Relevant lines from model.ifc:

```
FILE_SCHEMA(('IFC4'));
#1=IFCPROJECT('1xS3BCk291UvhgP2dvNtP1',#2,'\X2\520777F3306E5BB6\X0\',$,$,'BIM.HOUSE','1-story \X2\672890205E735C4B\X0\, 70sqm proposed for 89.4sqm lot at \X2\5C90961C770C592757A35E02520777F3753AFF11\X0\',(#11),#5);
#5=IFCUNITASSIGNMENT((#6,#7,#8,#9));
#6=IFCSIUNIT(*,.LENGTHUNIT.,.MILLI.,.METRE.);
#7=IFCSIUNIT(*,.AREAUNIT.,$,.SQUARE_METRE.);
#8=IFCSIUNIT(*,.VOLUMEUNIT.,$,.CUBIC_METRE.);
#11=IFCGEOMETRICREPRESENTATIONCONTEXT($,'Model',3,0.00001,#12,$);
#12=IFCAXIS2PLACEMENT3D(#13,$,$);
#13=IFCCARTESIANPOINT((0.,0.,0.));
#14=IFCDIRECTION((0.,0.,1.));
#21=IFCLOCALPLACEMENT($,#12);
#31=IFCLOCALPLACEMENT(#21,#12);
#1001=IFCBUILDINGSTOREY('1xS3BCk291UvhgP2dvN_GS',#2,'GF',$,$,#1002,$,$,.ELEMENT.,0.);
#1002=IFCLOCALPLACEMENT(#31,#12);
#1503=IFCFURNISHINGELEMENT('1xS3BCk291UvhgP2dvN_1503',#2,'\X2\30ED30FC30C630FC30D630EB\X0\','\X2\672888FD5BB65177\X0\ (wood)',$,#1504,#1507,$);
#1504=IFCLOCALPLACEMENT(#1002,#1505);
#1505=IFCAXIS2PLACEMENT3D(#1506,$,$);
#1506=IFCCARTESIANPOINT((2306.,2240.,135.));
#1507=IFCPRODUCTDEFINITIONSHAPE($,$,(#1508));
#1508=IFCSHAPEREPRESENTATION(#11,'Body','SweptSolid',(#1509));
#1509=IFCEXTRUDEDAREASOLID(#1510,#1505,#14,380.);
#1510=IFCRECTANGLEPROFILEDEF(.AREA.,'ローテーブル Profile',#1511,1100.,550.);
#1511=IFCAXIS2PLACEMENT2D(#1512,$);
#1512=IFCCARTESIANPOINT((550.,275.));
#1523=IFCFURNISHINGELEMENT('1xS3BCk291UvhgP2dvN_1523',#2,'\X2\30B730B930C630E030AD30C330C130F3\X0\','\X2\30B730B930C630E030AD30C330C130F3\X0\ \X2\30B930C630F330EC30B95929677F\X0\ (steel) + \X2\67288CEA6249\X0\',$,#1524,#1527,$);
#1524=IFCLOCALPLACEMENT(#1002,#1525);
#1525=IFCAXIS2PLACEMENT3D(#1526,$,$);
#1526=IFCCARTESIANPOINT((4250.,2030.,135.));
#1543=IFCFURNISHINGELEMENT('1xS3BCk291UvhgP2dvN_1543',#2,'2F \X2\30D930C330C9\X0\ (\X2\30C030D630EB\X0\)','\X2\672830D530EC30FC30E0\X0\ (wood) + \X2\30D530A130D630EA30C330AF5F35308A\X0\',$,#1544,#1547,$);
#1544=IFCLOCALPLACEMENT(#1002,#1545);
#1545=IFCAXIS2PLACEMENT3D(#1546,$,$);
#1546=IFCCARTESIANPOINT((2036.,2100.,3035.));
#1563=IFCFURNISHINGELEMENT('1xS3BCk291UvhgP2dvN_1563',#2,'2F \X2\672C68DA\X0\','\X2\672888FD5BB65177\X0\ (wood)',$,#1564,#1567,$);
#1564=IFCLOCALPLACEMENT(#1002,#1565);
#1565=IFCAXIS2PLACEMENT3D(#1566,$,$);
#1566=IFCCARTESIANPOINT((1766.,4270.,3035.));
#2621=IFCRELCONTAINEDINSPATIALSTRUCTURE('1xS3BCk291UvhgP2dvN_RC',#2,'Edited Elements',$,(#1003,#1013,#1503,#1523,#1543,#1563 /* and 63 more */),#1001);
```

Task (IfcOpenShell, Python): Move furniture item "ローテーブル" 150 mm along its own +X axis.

```python
import ifcopenshell
import ifcopenshell.api.geometry
import ifcopenshell.util.placement
import ifcopenshell.util.unit

model = ifcopenshell.open("model.ifc")
unit_scale = ifcopenshell.util.unit.calculate_unit_scale(model)

item = model.by_guid("1xS3BCk291UvhgP2dvN_1503")
matrix = ifcopenshell.util.placement.get_local_placement(item.ObjectPlacement)
matrix[:3, 3] += matrix[:3, 0] * 0.15 / unit_scale
ifcopenshell.api.geometry.edit_object_placement(model, product=item, matrix=matrix, is_si=False)

print(ifcopenshell.util.placement.get_local_placement(item.ObjectPlacement).round(3) + 0.0)

model.write("model-out.ifc")
```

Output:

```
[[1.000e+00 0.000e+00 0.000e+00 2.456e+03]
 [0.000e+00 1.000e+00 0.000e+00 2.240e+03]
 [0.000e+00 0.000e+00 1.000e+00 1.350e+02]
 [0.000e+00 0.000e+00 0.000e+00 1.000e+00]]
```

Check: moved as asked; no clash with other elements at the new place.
